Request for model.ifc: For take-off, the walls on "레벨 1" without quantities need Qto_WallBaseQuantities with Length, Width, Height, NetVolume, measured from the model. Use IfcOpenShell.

First a look at what the model holds.

```python
import ifcopenshell
import ifcopenshell.util.element
import ifcopenshell.util.unit

model = ifcopenshell.open("model.ifc")
print(model.schema)
for unit_type in ("LENGTHUNIT", "AREAUNIT", "VOLUMEUNIT"):
    print(unit_type, ifcopenshell.util.unit.calculate_unit_scale(model, unit_type))
storey = next(s for s in model.by_type("IfcBuildingStorey") if s.Name == "레벨 1")
walls = [e for e in ifcopenshell.util.element.get_decomposition(storey) if e.is_a("IfcWall")]
for e in sorted(walls, key=lambda e: e.id()):
    print(e.id(), e.is_a(), e.Name, list(ifcopenshell.util.element.get_psets(e, qtos_only=True)), sep=" | ")
```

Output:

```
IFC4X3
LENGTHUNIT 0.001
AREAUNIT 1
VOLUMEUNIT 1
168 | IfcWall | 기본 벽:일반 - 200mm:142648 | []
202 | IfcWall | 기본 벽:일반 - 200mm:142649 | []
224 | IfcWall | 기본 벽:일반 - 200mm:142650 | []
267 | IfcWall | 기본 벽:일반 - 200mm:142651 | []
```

```python
import ifcopenshell
import ifcopenshell.api.pset
import ifcopenshell.geom
import ifcopenshell.util.element
import ifcopenshell.util.shape
import ifcopenshell.util.unit

model = ifcopenshell.open("model.ifc")
unit_scale = ifcopenshell.util.unit.calculate_unit_scale(model)
volume_scale = ifcopenshell.util.unit.calculate_unit_scale(model, "VOLUMEUNIT")
settings = ifcopenshell.geom.settings()

storey = next(s for s in model.by_type("IfcBuildingStorey") if s.Name == "레벨 1")
walls = [e for e in ifcopenshell.util.element.get_decomposition(storey) if e.is_a("IfcWall")]

for e in sorted(walls, key=lambda e: e.id()):
    if ifcopenshell.util.element.get_psets(e, qtos_only=True, should_inherit=False):
        continue
    # Geometry comes back in metres, in the element's own axes.
    shape = ifcopenshell.geom.create_shape(settings, e)
    values = {
        "Length": ifcopenshell.util.shape.get_x(shape.geometry) / unit_scale,
        "Width": ifcopenshell.util.shape.get_y(shape.geometry) / unit_scale,
        "Height": ifcopenshell.util.shape.get_z(shape.geometry) / unit_scale,
        "NetVolume": ifcopenshell.util.shape.get_volume(shape.geometry) / volume_scale,
    }
    qto = ifcopenshell.api.pset.add_qto(model, product=e, name="Qto_WallBaseQuantities")
    ifcopenshell.api.pset.edit_qto(model, qto=qto, properties=values)
    print(e.id(), {k: round(v, 3) for k, v in values.items()})

model.write("model_v2.ifc")
```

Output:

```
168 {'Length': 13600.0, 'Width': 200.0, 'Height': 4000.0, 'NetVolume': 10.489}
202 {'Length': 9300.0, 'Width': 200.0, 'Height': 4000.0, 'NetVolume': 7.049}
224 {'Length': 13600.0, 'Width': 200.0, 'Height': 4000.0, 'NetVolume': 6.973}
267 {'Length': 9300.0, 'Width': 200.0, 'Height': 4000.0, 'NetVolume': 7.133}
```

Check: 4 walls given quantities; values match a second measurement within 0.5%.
